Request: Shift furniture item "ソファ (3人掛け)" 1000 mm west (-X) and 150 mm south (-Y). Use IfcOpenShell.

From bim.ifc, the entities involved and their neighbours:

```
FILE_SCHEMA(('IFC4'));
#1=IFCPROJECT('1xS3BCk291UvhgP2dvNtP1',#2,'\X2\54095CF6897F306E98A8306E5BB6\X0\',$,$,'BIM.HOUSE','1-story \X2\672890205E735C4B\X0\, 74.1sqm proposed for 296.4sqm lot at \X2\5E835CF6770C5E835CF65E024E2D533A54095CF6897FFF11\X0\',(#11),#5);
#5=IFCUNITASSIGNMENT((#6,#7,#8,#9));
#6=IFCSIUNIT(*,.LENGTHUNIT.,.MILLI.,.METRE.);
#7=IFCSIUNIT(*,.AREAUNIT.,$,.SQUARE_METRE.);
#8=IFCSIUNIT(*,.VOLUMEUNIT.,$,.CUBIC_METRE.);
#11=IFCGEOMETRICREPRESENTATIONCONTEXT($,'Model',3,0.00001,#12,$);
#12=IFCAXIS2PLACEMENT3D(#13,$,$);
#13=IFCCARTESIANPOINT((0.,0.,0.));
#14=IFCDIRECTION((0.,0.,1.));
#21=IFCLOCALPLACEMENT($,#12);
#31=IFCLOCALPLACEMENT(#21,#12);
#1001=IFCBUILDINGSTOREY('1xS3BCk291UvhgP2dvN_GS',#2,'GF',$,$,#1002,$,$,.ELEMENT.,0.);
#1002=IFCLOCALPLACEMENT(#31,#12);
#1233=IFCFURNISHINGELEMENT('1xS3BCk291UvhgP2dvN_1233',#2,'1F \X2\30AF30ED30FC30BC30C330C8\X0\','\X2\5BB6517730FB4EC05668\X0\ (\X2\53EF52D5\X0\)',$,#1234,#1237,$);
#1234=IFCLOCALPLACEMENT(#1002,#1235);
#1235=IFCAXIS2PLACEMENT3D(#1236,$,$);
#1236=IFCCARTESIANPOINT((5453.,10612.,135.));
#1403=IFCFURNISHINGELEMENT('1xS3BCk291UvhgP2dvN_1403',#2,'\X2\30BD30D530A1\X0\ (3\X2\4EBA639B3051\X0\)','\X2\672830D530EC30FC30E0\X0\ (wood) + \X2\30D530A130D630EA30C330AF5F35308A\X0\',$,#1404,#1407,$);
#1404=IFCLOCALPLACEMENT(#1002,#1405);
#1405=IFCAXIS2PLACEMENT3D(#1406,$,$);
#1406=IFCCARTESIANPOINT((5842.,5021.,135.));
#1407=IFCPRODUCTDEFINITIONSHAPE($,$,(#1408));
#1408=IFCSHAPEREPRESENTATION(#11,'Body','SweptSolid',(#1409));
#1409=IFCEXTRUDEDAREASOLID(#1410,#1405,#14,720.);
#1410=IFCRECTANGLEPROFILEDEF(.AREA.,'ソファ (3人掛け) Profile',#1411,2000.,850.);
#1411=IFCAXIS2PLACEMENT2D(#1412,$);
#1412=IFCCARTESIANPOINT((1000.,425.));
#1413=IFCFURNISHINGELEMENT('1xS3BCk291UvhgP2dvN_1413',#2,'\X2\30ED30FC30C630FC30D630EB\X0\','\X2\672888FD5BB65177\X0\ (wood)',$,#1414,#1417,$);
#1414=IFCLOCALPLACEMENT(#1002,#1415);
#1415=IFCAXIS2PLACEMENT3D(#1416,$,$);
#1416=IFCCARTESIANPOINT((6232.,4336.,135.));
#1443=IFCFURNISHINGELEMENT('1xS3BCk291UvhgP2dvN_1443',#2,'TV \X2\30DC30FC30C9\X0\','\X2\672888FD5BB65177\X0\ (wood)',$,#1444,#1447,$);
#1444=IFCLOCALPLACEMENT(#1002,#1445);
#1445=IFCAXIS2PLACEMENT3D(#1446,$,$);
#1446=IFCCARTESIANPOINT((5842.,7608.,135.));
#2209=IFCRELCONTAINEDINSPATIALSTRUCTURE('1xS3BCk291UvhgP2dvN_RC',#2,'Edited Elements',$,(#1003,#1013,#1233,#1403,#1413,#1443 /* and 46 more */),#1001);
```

```python
import ifcopenshell
import ifcopenshell.api.geometry
import ifcopenshell.util.placement
import ifcopenshell.util.unit

model = ifcopenshell.open("bim.ifc")
unit_scale = ifcopenshell.util.unit.calculate_unit_scale(model)

item = model.by_guid("1xS3BCk291UvhgP2dvN_1403")
matrix = ifcopenshell.util.placement.get_local_placement(item.ObjectPlacement)
matrix[0, 3] -= 1 / unit_scale
matrix[1, 3] -= 0.15 / unit_scale
ifcopenshell.api.geometry.edit_object_placement(model, product=item, matrix=matrix, is_si=False)

print(ifcopenshell.util.placement.get_local_placement(item.ObjectPlacement).round(3) + 0.0)

model.write("bim_v2.ifc")
```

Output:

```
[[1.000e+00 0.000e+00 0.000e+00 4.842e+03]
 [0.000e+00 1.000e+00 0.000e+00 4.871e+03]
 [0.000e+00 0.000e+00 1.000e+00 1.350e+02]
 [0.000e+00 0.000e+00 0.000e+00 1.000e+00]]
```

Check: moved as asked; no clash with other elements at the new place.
